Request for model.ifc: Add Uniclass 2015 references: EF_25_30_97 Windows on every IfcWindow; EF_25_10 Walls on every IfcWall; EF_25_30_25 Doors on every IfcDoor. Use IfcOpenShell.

First a look at what the model holds.

```python
import ifcopenshell

model = ifcopenshell.open("model.ifc")
print(model.schema)
print("classifications:", [c.Name for c in model.by_type("IfcClassification")])
for ifc_class in ("IfcDoor", "IfcRoof", "IfcStair", "IfcWall", "IfcWindow"):
    print(ifc_class, len(model.by_type(ifc_class)))
```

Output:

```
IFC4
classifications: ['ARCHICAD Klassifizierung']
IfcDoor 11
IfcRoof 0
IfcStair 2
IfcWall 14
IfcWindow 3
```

```python
import ifcopenshell
import ifcopenshell.api.classification

model = ifcopenshell.open("model.ifc")

system = ifcopenshell.api.classification.add_classification(model, classification="Uniclass 2015")

codes = {
    "IfcWindow": ("EF_25_30_97", "Windows"),
    "IfcWall": ("EF_25_10", "Walls"),
    "IfcDoor": ("EF_25_30_25", "Doors"),
}
for ifc_class, (code, name) in codes.items():
    products = model.by_type(ifc_class)
    ifcopenshell.api.classification.add_reference(
        model, products=products, classification=system, identification=code, name=name
    )
    print(code, len(products))

model.write("model_edited.ifc")
```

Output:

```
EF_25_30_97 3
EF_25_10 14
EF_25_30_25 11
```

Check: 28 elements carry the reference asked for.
